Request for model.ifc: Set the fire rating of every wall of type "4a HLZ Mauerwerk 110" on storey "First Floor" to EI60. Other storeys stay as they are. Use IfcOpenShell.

First a look at what the model holds.

```python
import ifcopenshell
import ifcopenshell.util.element

model = ifcopenshell.open("model.ifc")
print(model.schema)
storey = next(s for s in model.by_type("IfcBuildingStorey") if s.Name == "First Floor")
walls = [e for e in ifcopenshell.util.element.get_decomposition(storey) if e.is_a("IfcWall")]
seen = {}
for e in walls:
    element_type = ifcopenshell.util.element.get_type(e)
    key = (element_type.Name if element_type != e and element_type else None, ifcopenshell.util.element.get_pset(e, "Pset_WallCommon", "FireRating"))
    seen[key] = seen.get(key, 0) + 1
for (name, value), count in sorted(seen.items(), key=str):
    print(count, "x", name, "|", value)
```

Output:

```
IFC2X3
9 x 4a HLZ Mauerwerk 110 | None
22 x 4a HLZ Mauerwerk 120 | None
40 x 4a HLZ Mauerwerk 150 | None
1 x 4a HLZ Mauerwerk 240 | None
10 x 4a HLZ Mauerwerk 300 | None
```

```python
import ifcopenshell
import ifcopenshell.api.pset
import ifcopenshell.util.element

model = ifcopenshell.open("model.ifc")

storey = next(s for s in model.by_type("IfcBuildingStorey") if s.Name == "First Floor")
walls = [e for e in ifcopenshell.util.element.get_decomposition(storey) if e.is_a("IfcWall")]

count = 0
for e in walls:
    element_type = ifcopenshell.util.element.get_type(e)
    if element_type in (None, e) or element_type.Name != "4a HLZ Mauerwerk 110":
        continue
    # add_pset returns the element's existing set when there is one.
    pset = ifcopenshell.api.pset.add_pset(model, product=e, name="Pset_WallCommon")
    ifcopenshell.api.pset.edit_pset(model, pset=pset, properties={"FireRating": "EI60"})
    count += 1

print(count, "walls updated")

model.write("model_v2.ifc")
```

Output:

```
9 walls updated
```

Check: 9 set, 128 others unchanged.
